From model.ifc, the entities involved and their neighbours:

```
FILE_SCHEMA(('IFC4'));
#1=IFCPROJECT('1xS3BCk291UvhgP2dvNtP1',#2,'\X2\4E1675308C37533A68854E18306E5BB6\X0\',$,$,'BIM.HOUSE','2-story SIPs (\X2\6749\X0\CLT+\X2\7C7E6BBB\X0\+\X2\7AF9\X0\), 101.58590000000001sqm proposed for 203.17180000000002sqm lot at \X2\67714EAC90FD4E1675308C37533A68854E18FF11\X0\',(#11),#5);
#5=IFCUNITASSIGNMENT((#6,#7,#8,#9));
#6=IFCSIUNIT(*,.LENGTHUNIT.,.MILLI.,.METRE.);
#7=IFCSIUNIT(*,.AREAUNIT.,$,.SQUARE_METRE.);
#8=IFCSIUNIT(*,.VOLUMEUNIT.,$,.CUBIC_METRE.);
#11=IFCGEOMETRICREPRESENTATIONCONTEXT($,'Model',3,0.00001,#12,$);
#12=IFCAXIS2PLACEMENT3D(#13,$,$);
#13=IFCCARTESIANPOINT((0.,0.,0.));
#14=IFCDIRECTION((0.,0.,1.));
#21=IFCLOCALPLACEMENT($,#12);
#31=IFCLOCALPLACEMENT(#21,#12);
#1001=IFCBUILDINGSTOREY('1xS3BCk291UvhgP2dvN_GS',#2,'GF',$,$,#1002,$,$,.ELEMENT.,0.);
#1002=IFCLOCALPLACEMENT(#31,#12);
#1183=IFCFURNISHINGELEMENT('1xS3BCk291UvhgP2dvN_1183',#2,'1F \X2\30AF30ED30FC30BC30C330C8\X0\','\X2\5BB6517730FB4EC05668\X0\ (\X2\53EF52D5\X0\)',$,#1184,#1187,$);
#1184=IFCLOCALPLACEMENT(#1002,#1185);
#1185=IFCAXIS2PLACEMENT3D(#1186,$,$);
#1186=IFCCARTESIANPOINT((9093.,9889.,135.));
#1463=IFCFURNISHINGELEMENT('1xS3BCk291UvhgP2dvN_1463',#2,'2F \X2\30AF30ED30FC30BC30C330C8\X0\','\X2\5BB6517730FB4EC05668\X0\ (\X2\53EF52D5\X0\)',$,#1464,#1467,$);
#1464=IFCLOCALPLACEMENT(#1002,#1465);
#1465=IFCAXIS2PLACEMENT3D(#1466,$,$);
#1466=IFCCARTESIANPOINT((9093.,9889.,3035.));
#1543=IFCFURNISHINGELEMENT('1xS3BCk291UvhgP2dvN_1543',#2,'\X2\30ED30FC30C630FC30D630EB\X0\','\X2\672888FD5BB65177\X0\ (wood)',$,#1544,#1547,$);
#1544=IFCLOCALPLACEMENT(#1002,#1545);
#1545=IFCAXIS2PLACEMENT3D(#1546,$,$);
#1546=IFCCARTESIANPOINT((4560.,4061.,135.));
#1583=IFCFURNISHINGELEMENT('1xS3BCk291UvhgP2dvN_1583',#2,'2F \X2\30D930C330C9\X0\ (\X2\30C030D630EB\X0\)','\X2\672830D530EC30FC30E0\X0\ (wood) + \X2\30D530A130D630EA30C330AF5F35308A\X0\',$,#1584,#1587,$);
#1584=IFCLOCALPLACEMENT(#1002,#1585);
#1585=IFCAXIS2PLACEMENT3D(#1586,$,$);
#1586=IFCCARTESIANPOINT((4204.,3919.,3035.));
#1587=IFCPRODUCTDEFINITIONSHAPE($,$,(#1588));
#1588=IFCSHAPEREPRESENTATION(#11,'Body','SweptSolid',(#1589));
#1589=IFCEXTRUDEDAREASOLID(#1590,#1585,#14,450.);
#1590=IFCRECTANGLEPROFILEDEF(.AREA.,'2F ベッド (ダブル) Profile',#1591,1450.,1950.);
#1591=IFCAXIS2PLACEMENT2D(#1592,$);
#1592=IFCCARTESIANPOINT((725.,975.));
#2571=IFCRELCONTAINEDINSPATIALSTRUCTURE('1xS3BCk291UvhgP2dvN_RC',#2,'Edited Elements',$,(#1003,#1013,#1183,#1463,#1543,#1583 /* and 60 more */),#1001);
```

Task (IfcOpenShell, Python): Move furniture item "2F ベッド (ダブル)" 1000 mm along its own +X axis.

```python
import ifcopenshell
import ifcopenshell.api.geometry
import ifcopenshell.util.placement

model = ifcopenshell.open("model.ifc")

item = model.by_guid("1xS3BCk291UvhgP2dvN_1583")
matrix = ifcopenshell.util.placement.get_local_placement(item.ObjectPlacement)
matrix[:3, 3] += matrix[:3, 0] * 1000.0
ifcopenshell.api.geometry.edit_object_placement(model, product=item, matrix=matrix, is_si=False)

print(ifcopenshell.util.placement.get_local_placement(item.ObjectPlacement).round(3) + 0.0)

model.write("model_v2.ifc")
```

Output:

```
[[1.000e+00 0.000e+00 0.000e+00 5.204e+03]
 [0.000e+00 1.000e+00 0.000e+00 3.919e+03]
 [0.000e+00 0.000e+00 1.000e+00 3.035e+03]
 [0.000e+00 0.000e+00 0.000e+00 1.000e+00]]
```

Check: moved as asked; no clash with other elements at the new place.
